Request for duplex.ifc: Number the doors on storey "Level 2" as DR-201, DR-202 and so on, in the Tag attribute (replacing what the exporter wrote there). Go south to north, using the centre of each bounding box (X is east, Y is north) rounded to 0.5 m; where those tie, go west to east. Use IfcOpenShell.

First a look at what the model holds.

```python
import ifcopenshell
import ifcopenshell.util.element
import ifcopenshell.util.placement

model = ifcopenshell.open("duplex.ifc")
print(model.schema)
storey = next(s for s in model.by_type("IfcBuildingStorey") if s.Name == "Level 2")
doors = [e for e in ifcopenshell.util.element.get_decomposition(storey) if e.is_a("IfcDoor")]
for e in sorted(doors, key=lambda e: e.id()):
    origin = ifcopenshell.util.placement.get_local_placement(e.ObjectPlacement)[:3, 3]
    print(e.id(), e.Tag, e.Name, origin.round(2) + 0.0, sep=" | ")
```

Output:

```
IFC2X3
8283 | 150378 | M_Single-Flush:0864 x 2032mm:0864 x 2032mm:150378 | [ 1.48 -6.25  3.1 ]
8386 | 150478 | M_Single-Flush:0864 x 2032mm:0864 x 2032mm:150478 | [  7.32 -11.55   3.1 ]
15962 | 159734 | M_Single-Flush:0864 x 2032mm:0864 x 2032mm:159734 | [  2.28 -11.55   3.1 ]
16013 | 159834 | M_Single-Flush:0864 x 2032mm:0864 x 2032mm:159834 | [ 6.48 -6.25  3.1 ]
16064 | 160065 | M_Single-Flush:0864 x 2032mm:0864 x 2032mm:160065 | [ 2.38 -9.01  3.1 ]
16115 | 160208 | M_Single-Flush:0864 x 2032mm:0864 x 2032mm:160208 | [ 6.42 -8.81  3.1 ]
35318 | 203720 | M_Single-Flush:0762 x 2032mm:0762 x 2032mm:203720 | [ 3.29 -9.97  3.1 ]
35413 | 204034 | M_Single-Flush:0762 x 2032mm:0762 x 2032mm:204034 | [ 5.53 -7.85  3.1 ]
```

```python
import ifcopenshell
import ifcopenshell.geom
import ifcopenshell.util.element
import ifcopenshell.util.shape

model = ifcopenshell.open("duplex.ifc")
settings = ifcopenshell.geom.settings()
settings.set("use-world-coords", True)


def centre(element):
    shape = ifcopenshell.geom.create_shape(settings, element)
    return ifcopenshell.util.shape.get_bbox_centroid(shape.geometry)


storey = next(s for s in model.by_type("IfcBuildingStorey") if s.Name == "Level 2")
doors = [e for e in ifcopenshell.util.element.get_decomposition(storey) if e.is_a("IfcDoor")]

# Insertion points can sit at a corner or the storey origin, so sort by the geometry (in metres).
centres = {e: centre(e) for e in doors}
doors.sort(key=lambda e: (round(centres[e][1] / 0.5), centres[e][0]))

for i, e in enumerate(doors, start=1):
    number = f"DR-2{i:02d}"
    e.Tag = number
    print(e.id(), number)

model.write("duplex_updated.ifc")
```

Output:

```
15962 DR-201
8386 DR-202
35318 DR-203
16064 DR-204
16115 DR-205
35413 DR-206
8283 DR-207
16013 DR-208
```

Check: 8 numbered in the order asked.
